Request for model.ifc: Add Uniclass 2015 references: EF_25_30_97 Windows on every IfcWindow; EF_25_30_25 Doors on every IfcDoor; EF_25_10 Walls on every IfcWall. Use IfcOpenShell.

First a look at what the model holds.

```python
import ifcopenshell

model = ifcopenshell.open("model.ifc")
print(model.schema)
print("classifications:", [c.Name for c in model.by_type("IfcClassification")])
for ifc_class in ("IfcDoor", "IfcRoof", "IfcStair", "IfcWall", "IfcWindow"):
    print(ifc_class, len(model.by_type(ifc_class)))
```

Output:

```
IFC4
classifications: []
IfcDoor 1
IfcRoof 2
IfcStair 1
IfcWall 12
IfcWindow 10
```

```python
import ifcopenshell
import ifcopenshell.api.classification

model = ifcopenshell.open("model.ifc")

system = ifcopenshell.api.classification.add_classification(model, classification="Uniclass 2015")

codes = {
    "IfcWindow": ("EF_25_30_97", "Windows"),
    "IfcDoor": ("EF_25_30_25", "Doors"),
    "IfcWall": ("EF_25_10", "Walls"),
}
for ifc_class, (code, name) in codes.items():
    products = model.by_type(ifc_class)
    ifcopenshell.api.classification.add_reference(
        model, products=products, classification=system, identification=code, name=name
    )
    print(code, len(products))

model.write("model-out.ifc")
```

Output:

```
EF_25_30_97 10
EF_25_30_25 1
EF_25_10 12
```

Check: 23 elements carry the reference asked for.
